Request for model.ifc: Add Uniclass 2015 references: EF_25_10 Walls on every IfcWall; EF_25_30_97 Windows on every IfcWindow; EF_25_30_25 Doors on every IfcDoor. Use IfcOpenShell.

First a look at what the model holds.

```python
import ifcopenshell

model = ifcopenshell.open("model.ifc")
print(model.schema)
print("classifications:", [c.Name for c in model.by_type("IfcClassification")])
for ifc_class in ("IfcDoor", "IfcRoof", "IfcStair", "IfcWall", "IfcWindow"):
    print(ifc_class, len(model.by_type(ifc_class)))
```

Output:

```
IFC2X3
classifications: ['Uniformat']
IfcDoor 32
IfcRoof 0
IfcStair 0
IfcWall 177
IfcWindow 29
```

```python
import ifcopenshell
import ifcopenshell.api.classification

model = ifcopenshell.open("model.ifc")

# IFC2X3 requires Source and Edition and has no link from the project to the system.
system = model.create_entity("IfcClassification", Source="NBS", Edition="2015", Name="Uniclass 2015")

codes = {
    "IfcWall": ("EF_25_10", "Walls"),
    "IfcWindow": ("EF_25_30_97", "Windows"),
    "IfcDoor": ("EF_25_30_25", "Doors"),
}
for ifc_class, (code, name) in codes.items():
    products = model.by_type(ifc_class)
    ifcopenshell.api.classification.add_reference(
        model, products=products, classification=system, identification=code, name=name
    )
    print(code, len(products))

model.write("model-out.ifc")
```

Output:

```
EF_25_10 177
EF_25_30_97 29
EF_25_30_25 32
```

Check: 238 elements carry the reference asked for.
